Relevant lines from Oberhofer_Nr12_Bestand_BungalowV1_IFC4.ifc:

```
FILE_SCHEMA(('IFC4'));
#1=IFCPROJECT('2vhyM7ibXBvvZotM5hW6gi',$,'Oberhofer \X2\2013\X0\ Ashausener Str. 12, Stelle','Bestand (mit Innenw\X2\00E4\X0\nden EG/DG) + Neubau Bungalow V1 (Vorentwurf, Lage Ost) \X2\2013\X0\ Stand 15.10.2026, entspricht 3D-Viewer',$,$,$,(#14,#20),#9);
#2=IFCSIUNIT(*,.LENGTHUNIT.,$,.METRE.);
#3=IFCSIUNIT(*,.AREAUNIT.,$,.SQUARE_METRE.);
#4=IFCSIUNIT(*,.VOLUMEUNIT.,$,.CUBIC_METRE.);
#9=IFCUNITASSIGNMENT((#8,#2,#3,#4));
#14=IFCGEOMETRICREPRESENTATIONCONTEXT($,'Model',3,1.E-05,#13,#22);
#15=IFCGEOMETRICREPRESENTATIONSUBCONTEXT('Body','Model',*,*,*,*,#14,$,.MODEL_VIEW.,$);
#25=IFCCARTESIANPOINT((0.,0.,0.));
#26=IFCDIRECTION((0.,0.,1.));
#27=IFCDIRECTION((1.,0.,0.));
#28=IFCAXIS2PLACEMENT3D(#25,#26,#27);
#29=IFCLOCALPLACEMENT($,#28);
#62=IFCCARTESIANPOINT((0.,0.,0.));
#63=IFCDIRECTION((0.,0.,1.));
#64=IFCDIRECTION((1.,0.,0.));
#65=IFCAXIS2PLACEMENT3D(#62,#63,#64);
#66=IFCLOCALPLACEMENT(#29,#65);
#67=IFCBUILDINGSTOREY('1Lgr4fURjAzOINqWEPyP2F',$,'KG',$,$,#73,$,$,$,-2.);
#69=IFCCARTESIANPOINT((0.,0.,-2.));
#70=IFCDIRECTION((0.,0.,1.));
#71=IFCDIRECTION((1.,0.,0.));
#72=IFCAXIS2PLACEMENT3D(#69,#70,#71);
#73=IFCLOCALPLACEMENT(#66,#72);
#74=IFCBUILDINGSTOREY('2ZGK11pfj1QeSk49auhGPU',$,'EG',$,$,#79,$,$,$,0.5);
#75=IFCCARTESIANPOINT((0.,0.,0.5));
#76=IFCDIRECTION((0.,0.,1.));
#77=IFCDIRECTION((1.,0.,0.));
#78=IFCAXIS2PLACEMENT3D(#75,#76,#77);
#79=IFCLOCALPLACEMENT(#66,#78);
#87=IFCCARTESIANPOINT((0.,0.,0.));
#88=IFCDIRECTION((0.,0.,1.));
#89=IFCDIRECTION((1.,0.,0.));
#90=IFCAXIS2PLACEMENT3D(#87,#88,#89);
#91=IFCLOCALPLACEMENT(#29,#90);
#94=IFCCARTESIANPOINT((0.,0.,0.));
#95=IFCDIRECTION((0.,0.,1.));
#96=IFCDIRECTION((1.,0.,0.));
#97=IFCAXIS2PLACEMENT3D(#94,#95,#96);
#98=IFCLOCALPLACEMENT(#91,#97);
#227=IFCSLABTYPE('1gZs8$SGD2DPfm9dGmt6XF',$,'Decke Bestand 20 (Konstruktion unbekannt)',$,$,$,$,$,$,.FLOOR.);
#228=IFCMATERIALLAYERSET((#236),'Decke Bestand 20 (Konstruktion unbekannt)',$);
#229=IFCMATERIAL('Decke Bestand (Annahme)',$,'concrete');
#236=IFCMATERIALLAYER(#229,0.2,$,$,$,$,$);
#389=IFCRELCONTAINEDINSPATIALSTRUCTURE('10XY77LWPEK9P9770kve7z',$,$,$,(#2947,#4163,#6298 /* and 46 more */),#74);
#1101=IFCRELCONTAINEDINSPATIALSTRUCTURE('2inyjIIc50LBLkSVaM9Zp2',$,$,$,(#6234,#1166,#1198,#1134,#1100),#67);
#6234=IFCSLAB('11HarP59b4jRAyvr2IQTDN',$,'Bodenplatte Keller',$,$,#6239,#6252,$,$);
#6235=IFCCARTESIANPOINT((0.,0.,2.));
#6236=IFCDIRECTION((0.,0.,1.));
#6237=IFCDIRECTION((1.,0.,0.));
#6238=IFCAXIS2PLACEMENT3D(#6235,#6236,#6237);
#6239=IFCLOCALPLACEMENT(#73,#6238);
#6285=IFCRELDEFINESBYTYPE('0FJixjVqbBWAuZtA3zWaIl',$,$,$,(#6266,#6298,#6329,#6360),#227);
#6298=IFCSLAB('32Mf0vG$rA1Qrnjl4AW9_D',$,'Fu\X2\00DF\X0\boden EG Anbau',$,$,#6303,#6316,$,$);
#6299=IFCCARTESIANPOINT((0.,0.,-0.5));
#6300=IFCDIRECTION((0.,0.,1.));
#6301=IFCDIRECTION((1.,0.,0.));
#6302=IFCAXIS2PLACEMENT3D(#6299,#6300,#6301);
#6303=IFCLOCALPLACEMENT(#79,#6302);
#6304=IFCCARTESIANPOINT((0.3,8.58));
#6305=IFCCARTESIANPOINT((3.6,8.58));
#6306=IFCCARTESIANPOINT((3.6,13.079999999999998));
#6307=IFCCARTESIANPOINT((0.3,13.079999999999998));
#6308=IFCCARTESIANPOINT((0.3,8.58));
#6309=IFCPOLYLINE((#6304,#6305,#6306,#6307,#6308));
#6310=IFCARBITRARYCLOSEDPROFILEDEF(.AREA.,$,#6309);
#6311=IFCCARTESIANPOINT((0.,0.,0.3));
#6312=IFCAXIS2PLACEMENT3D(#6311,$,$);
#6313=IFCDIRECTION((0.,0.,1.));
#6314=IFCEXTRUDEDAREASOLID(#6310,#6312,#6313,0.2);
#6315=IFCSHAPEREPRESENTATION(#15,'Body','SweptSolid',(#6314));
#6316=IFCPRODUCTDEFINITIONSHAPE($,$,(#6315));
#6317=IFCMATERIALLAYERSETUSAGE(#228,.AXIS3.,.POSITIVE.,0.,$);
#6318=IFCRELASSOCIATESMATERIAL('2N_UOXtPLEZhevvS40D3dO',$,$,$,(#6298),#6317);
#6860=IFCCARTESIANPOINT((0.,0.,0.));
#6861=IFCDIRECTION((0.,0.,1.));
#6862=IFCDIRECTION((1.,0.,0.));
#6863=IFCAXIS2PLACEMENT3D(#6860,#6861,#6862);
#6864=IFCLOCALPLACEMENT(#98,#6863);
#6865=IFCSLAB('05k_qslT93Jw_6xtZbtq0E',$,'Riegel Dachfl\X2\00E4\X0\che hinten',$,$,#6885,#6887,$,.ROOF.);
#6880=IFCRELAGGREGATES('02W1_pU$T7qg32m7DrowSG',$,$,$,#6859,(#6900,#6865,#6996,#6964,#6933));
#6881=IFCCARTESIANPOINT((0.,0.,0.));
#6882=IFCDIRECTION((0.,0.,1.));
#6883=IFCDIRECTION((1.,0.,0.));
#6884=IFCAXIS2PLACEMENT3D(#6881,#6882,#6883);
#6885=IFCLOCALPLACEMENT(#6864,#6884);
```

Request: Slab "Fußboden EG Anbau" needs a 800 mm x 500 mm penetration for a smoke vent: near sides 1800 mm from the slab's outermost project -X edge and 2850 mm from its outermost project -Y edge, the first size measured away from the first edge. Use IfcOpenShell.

```python
import numpy as np
import ifcopenshell
import ifcopenshell.api.feature
import ifcopenshell.api.geometry
import ifcopenshell.api.root
import ifcopenshell.geom
import ifcopenshell.util.placement
import ifcopenshell.util.representation
import ifcopenshell.util.shape
import ifcopenshell.util.unit

model = ifcopenshell.open("Oberhofer_Nr12_Bestand_BungalowV1_IFC4.ifc")
unit_scale = ifcopenshell.util.unit.calculate_unit_scale(model)
settings = ifcopenshell.geom.settings()


def volume(element):
    """Net volume in cubic metres, openings subtracted."""
    shape = ifcopenshell.geom.create_shape(settings, element)
    return ifcopenshell.util.shape.get_volume(shape.geometry)


slab = model.by_guid("32Mf0vG$rA1Qrnjl4AW9_D")
before = volume(slab)

# Extent in the slab's own axes, in metres. The edges named are its -X and -Y sides.
slab_shape = ifcopenshell.geom.create_shape(settings, slab)
vertices = ifcopenshell.util.shape.get_vertices(slab_shape.geometry)
x_min, y_min, bottom = vertices.min(axis=0)
top = vertices[:, 2].max()

opening = ifcopenshell.api.root.create_entity(model, ifc_class="IfcOpeningElement", name="Smoke vent opening", predefined_type="OPENING")
context = ifcopenshell.util.representation.get_context(model, "Model", "Body", "MODEL_VIEW")
width, depth = 0.8, 0.5
outline = [(0.0, 0.0), (width, 0.0), (width, depth), (0.0, depth), (0.0, 0.0)]
# Overshoot both faces by 50 mm so the cut is clean.
shape = ifcopenshell.api.geometry.add_slab_representation(
    model, context=context, depth=top - bottom + 0.1, polyline=outline
)
ifcopenshell.api.geometry.assign_representation(model, product=opening, representation=shape)

matrix = ifcopenshell.util.placement.get_local_placement(slab.ObjectPlacement)
matrix[:, 3] = matrix @ np.append(np.array([x_min + 1.8, y_min + 2.85, bottom - 0.05]) / unit_scale, 1.0)
ifcopenshell.api.geometry.edit_object_placement(model, product=opening, matrix=matrix, is_si=False)
ifcopenshell.api.feature.add_feature(model, feature=opening, element=slab)

after = volume(slab)

print(f"slab volume {before:.3f} -> {after:.3f} m3")

model.write("Oberhofer_Nr12_Bestand_BungalowV1_IFC4_edited.ifc")
```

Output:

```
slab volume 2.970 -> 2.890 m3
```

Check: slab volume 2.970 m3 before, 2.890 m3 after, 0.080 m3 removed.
